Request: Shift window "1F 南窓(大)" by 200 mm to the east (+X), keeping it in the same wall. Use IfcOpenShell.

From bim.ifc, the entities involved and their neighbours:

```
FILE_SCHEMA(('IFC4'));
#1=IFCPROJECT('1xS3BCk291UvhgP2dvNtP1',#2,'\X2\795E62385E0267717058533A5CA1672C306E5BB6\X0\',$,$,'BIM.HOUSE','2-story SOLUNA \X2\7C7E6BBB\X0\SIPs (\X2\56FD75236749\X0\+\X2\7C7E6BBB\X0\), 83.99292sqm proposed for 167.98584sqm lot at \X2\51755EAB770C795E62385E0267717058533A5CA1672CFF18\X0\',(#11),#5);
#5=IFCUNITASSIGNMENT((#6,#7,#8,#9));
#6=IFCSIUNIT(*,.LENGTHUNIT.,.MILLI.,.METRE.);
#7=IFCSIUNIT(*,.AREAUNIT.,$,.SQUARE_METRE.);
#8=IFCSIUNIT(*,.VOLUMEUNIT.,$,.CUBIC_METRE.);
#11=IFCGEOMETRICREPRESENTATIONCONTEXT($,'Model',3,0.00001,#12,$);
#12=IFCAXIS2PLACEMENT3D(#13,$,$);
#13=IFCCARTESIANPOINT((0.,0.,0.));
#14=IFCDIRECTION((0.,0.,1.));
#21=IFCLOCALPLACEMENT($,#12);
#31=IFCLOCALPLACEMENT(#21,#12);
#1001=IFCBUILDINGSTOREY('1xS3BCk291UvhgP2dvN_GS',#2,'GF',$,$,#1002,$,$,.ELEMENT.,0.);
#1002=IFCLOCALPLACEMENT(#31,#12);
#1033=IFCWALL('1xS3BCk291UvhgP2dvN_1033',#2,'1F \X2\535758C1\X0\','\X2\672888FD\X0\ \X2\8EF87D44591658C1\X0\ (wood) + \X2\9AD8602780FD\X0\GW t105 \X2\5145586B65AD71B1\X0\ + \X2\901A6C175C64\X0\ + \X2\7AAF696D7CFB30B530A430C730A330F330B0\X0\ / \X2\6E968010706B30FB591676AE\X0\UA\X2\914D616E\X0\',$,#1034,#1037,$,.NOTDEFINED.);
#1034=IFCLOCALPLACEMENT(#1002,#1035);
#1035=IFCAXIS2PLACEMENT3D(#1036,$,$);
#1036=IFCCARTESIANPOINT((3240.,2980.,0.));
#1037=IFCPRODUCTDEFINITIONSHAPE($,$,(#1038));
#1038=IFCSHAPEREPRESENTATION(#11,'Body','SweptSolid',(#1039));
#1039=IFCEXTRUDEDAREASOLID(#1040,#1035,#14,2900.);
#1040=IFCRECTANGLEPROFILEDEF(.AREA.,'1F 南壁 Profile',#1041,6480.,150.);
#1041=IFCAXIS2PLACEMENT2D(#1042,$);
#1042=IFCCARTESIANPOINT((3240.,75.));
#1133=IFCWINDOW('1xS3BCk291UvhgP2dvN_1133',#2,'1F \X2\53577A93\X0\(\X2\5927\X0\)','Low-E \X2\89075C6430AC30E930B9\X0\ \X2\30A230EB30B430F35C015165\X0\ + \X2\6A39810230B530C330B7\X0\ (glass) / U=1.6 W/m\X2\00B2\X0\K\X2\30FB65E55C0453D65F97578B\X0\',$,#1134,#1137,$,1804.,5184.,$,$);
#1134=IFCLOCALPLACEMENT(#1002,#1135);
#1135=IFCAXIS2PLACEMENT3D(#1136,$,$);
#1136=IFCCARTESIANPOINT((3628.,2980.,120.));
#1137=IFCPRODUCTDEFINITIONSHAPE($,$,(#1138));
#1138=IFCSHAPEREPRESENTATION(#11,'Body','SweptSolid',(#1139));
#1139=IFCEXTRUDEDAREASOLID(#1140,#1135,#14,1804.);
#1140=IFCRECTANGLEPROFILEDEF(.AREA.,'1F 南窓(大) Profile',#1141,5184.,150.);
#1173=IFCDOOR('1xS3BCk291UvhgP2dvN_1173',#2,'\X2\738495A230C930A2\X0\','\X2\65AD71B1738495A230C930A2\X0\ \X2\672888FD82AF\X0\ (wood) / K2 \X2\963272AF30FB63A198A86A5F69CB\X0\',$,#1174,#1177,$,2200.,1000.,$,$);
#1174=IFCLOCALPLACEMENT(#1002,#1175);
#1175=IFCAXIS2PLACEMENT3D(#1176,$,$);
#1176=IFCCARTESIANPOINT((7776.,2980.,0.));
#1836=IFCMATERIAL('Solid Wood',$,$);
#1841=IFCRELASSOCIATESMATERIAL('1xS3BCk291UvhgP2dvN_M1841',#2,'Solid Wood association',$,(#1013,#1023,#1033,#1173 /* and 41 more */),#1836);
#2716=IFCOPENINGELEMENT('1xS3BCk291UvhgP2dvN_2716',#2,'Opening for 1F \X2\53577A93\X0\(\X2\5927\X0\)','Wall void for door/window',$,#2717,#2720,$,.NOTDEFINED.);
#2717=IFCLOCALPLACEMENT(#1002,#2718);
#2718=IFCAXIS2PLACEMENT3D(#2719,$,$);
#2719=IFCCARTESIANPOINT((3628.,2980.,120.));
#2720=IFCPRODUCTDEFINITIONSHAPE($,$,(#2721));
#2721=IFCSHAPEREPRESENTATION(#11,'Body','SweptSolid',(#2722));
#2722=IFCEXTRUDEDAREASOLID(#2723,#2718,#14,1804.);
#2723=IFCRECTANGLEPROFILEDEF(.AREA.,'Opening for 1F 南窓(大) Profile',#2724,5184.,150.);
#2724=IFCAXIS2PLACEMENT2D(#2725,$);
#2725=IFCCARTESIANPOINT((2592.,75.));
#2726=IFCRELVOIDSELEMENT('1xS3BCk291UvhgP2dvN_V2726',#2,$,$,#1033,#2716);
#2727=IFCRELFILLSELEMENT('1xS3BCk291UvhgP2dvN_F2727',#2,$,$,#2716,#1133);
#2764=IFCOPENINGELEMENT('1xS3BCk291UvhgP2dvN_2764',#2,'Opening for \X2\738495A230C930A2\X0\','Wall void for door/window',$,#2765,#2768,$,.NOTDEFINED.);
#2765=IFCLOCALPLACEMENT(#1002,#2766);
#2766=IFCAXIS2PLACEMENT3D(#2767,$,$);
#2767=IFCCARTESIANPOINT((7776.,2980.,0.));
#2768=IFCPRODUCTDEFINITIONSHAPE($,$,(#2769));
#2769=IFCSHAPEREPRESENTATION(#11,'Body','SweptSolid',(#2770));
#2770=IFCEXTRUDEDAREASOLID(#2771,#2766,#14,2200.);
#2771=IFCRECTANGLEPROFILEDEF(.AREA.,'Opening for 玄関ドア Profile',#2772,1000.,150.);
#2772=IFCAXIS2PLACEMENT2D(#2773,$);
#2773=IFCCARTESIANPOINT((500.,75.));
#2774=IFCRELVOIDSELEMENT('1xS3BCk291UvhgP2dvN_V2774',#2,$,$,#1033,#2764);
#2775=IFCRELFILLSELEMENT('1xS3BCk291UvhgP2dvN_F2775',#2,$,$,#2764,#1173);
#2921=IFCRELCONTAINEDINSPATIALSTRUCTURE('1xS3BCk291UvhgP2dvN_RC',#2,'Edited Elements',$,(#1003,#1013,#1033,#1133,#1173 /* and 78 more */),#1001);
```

```python
import ifcopenshell
import ifcopenshell.api.geometry
import ifcopenshell.util.placement
import ifcopenshell.util.unit

model = ifcopenshell.open("bim.ifc")
unit_scale = ifcopenshell.util.unit.calculate_unit_scale(model)

window = model.by_guid("1xS3BCk291UvhgP2dvN_1133")
opening = window.FillsVoids[0].RelatingOpeningElement
wall = opening.VoidsElements[0].RelatingBuildingElement

wall_matrix = ifcopenshell.util.placement.get_local_placement(wall.ObjectPlacement)
shift = wall_matrix[:3, 0] * 0.2 / unit_scale
before = ifcopenshell.util.placement.get_local_placement(window.ObjectPlacement)[:3, 3].copy()

# The window is not placed relative to its opening, so move both.
for product in (opening, window):
    matrix = ifcopenshell.util.placement.get_local_placement(product.ObjectPlacement)
    matrix[:3, 3] += shift
    ifcopenshell.api.geometry.edit_object_placement(model, product=product, matrix=matrix, is_si=False)

after = ifcopenshell.util.placement.get_local_placement(window.ObjectPlacement)[:3, 3]
print("window moved by", (after - before).round(3) + 0.0)

model.write("bim_v2.ifc")
```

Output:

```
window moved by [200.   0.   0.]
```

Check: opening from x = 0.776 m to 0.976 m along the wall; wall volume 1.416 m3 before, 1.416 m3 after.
